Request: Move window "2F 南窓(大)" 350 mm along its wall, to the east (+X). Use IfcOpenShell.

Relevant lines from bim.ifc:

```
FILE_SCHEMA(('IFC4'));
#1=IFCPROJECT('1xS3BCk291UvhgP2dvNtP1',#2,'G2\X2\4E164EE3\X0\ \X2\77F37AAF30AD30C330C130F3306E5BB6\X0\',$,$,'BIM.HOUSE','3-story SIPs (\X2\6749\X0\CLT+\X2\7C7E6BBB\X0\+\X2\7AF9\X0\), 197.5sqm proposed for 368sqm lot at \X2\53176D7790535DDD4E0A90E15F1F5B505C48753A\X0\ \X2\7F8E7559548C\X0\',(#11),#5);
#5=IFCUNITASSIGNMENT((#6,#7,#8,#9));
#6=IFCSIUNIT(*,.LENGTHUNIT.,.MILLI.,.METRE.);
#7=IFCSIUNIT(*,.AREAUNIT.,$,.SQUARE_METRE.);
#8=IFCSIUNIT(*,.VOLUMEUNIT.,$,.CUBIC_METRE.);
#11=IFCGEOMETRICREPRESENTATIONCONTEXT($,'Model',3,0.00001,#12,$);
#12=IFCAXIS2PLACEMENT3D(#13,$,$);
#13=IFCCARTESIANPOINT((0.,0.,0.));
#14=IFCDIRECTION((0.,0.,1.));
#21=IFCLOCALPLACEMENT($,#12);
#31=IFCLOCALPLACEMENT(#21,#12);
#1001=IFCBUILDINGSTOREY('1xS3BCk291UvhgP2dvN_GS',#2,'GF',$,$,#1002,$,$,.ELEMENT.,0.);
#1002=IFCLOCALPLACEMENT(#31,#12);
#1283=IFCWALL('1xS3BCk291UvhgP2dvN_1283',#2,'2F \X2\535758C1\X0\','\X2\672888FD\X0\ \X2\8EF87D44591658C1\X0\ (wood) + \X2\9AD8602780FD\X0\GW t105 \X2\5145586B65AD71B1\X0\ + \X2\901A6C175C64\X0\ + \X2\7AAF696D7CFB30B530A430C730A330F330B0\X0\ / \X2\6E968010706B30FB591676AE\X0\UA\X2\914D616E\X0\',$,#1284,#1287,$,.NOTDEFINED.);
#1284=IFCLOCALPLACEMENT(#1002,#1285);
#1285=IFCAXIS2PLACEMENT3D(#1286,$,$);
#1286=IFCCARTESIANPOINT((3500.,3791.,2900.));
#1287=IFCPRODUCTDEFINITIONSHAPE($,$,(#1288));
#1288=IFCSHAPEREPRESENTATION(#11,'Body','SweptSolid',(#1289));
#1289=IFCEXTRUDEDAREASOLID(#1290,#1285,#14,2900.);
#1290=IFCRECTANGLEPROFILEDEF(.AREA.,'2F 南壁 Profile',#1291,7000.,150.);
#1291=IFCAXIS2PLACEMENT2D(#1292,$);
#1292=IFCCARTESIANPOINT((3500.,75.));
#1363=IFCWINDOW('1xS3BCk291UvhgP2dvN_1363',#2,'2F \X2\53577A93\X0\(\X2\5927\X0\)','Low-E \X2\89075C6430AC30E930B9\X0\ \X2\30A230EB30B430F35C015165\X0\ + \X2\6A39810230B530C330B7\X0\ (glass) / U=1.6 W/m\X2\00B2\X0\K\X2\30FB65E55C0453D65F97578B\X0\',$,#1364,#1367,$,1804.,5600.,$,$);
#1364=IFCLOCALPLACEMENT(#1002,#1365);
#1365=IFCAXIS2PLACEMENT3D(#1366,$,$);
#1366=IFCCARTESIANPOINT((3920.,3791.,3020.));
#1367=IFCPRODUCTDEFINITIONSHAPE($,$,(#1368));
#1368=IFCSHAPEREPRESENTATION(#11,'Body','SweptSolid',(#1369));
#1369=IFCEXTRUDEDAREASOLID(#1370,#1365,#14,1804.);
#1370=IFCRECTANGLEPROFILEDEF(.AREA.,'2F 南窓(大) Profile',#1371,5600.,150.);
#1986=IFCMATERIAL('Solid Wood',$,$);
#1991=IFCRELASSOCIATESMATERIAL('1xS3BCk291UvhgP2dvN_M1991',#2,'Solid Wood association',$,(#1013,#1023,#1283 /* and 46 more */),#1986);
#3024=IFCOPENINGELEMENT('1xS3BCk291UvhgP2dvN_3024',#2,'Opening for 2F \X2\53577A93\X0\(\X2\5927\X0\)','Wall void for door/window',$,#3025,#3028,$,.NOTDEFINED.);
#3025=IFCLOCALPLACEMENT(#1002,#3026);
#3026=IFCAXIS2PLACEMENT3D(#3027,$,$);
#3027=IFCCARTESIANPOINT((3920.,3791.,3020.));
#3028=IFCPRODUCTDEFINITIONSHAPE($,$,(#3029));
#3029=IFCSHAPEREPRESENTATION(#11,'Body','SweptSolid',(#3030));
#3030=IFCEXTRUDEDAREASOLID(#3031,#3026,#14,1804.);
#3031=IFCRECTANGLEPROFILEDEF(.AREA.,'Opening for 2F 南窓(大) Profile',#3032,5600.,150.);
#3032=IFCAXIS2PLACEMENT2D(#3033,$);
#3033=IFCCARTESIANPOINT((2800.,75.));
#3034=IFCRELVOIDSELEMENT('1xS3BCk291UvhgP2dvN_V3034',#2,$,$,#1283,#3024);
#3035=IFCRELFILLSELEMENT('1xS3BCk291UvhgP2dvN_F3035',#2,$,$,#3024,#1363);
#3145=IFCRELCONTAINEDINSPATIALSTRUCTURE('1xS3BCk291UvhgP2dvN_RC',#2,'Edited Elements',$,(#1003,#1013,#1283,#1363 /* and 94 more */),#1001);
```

```python
import ifcopenshell
import ifcopenshell.api.geometry
import ifcopenshell.util.placement

model = ifcopenshell.open("bim.ifc")

window = model.by_guid("1xS3BCk291UvhgP2dvN_1363")
opening = window.FillsVoids[0].RelatingOpeningElement
wall = opening.VoidsElements[0].RelatingBuildingElement

wall_matrix = ifcopenshell.util.placement.get_local_placement(wall.ObjectPlacement)
shift = wall_matrix[:3, 0] * 350.0
before = ifcopenshell.util.placement.get_local_placement(window.ObjectPlacement)[:3, 3].copy()

# The window is not placed relative to its opening, so move both.
for product in (opening, window):
    matrix = ifcopenshell.util.placement.get_local_placement(product.ObjectPlacement)
    matrix[:3, 3] += shift
    ifcopenshell.api.geometry.edit_object_placement(model, product=product, matrix=matrix, is_si=False)

after = ifcopenshell.util.placement.get_local_placement(window.ObjectPlacement)[:3, 3]
print("window moved by", (after - before).round(3) + 0.0)

model.write("bim-out.ifc")
```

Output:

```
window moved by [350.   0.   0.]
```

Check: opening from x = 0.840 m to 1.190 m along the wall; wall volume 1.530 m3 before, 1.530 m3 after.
